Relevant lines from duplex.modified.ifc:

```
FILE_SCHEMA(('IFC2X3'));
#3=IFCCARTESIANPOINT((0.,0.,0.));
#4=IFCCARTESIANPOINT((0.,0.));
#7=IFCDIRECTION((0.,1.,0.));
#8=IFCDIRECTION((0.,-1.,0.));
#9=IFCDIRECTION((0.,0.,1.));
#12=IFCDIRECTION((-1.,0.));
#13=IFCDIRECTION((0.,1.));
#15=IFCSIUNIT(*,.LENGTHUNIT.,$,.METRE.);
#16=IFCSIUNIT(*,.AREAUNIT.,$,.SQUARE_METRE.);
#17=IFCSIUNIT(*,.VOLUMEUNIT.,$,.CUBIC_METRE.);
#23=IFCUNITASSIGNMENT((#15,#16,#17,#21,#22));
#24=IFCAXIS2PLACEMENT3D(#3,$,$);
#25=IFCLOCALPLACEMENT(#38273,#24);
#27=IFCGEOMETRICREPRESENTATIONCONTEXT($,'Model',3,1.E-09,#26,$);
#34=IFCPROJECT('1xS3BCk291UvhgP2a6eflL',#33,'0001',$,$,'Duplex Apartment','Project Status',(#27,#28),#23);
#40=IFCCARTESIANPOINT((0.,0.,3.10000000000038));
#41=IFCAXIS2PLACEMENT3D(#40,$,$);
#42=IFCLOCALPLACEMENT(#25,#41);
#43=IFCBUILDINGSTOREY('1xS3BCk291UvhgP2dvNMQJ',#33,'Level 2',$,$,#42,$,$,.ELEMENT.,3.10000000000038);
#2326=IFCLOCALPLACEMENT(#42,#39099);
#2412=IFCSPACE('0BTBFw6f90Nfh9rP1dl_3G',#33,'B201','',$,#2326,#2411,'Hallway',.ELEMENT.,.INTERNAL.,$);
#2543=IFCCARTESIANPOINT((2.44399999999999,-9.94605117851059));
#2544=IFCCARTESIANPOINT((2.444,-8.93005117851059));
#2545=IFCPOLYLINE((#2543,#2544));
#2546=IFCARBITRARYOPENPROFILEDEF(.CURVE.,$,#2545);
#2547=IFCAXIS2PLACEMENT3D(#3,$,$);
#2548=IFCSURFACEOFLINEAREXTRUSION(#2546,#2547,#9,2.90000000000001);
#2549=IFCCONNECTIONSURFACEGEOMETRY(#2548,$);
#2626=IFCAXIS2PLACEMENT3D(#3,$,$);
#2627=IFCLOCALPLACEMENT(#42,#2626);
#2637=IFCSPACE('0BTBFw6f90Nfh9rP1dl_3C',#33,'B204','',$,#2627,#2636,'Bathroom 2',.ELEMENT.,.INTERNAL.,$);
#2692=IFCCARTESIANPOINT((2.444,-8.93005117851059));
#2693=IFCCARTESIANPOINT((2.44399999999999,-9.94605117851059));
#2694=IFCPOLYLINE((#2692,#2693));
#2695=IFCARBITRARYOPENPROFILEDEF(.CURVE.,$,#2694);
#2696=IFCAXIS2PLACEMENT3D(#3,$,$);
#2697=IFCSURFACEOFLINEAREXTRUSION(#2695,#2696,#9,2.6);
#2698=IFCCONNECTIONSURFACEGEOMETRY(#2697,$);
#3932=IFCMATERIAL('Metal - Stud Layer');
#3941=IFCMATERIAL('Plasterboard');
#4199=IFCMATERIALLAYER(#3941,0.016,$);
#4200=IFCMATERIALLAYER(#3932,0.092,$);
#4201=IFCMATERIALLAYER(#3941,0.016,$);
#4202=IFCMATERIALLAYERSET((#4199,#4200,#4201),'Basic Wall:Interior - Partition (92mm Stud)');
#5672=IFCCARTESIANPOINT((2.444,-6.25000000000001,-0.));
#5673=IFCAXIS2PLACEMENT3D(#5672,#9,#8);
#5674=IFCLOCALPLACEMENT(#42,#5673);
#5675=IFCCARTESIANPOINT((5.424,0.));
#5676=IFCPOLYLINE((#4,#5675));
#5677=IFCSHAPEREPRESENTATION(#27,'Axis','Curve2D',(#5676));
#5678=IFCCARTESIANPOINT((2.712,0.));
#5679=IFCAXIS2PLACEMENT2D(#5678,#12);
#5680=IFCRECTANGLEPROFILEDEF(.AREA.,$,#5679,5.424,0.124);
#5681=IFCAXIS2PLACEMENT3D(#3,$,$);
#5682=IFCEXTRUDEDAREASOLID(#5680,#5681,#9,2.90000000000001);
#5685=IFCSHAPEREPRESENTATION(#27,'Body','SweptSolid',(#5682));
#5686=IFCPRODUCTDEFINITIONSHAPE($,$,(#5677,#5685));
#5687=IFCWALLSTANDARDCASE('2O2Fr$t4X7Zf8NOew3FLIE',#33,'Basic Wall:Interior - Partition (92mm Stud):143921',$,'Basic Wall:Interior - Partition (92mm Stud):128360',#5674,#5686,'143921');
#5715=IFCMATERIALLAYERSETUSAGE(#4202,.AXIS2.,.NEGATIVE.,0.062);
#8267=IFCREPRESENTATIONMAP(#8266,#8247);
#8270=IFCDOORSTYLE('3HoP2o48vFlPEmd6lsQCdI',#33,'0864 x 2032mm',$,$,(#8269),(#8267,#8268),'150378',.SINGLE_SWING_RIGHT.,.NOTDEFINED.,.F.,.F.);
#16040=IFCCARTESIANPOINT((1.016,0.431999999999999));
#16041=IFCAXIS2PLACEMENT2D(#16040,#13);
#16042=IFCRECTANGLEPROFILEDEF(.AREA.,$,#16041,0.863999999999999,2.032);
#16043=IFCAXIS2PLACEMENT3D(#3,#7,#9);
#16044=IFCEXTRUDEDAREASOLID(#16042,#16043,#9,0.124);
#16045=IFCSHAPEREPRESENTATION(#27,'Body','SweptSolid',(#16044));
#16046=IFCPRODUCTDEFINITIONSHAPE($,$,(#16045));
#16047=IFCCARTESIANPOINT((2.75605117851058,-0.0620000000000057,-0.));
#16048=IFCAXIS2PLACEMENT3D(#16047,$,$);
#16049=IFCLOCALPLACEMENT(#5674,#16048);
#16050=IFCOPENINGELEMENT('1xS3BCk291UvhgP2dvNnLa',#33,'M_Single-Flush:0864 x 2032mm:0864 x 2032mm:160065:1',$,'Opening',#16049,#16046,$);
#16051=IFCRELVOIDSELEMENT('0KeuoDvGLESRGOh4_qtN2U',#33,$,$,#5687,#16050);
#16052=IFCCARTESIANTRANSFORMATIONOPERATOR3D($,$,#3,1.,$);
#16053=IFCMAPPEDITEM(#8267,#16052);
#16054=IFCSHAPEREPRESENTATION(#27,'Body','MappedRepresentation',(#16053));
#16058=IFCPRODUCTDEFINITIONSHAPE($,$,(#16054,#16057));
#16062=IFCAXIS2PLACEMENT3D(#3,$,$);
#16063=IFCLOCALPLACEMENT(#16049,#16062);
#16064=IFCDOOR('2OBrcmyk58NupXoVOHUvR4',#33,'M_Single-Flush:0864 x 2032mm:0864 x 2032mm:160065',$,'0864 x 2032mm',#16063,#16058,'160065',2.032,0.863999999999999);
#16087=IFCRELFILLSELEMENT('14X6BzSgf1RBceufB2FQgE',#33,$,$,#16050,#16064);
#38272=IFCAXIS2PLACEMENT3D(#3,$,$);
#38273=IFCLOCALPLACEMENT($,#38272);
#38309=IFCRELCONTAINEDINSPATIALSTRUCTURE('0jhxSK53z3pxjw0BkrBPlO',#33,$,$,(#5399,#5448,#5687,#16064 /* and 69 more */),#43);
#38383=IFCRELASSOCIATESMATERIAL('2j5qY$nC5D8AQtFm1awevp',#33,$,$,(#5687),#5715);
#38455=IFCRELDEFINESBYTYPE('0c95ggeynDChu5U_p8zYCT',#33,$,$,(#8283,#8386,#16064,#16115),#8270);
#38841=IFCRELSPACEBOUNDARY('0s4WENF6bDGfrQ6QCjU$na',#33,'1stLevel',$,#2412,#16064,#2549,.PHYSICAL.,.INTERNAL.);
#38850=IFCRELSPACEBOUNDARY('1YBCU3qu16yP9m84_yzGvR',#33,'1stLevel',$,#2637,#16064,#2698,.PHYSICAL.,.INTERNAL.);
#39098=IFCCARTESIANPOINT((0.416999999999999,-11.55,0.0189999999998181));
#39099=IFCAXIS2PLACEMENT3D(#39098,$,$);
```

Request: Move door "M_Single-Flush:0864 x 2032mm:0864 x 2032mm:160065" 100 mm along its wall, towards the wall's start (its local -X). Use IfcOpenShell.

```python
import numpy as np
import ifcopenshell
import ifcopenshell.api.geometry
import ifcopenshell.util.placement

model = ifcopenshell.open("duplex.modified.ifc")

door = model.by_id(16064)
opening = door.FillsVoids[0].RelatingOpeningElement
wall = opening.VoidsElements[0].RelatingBuildingElement

wall_matrix = ifcopenshell.util.placement.get_local_placement(wall.ObjectPlacement)
shift = wall_matrix[:3, 0] * -0.1
before = ifcopenshell.util.placement.get_local_placement(door.ObjectPlacement)[:3, 3].copy()

# The door is placed relative to its opening, so it follows when the opening moves.
matrix = ifcopenshell.util.placement.get_local_placement(opening.ObjectPlacement)
matrix[:3, 3] += shift
ifcopenshell.api.geometry.edit_object_placement(
    model, product=opening, matrix=matrix, is_si=False, should_transform_children=True
)

# Space boundary surfaces are stored in each space's coordinates; move them too.
for rel in door.ProvidesBoundaries:
    if not rel.ConnectionGeometry:
        continue
    surface = rel.ConnectionGeometry.SurfaceOnRelatingElement
    space_matrix = ifcopenshell.util.placement.get_local_placement(rel.RelatingSpace.ObjectPlacement)
    point = np.array(surface.Position.Location.Coordinates) + space_matrix[:3, :3].T @ shift
    surface.Position = model.createIfcAxis2Placement3D(
        model.createIfcCartesianPoint(point.tolist()), surface.Position.Axis, surface.Position.RefDirection
    )

after = ifcopenshell.util.placement.get_local_placement(door.ObjectPlacement)[:3, 3]
print("door moved by", (after - before).round(3) + 0.0)

model.write("duplex.modified-out.ifc")
```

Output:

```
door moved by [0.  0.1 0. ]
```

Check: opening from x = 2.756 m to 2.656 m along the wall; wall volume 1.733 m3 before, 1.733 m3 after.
